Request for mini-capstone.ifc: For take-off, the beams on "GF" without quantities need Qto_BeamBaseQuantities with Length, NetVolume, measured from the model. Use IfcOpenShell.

First a look at what the model holds.

```python
import ifcopenshell
import ifcopenshell.util.element
import ifcopenshell.util.unit

model = ifcopenshell.open("mini-capstone.ifc")
print(model.schema)
for unit_type in ("LENGTHUNIT", "AREAUNIT", "VOLUMEUNIT"):
    print(unit_type, ifcopenshell.util.unit.calculate_unit_scale(model, unit_type))
storey = next(s for s in model.by_type("IfcBuildingStorey") if s.Name == "GF")
beams = [e for e in ifcopenshell.util.element.get_decomposition(storey) if e.is_a("IfcBeam")]
for e in sorted(beams, key=lambda e: e.id()):
    print(e.id(), e.is_a(), e.Name, list(ifcopenshell.util.element.get_psets(e, qtos_only=True)), sep=" | ")
```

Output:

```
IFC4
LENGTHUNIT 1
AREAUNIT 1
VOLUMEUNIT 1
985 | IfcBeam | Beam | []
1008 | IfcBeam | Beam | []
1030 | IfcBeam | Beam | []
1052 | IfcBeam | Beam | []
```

```python
import ifcopenshell
import ifcopenshell.api.pset
import ifcopenshell.geom
import ifcopenshell.util.element
import ifcopenshell.util.shape
import ifcopenshell.util.unit

model = ifcopenshell.open("mini-capstone.ifc")
unit_scale = ifcopenshell.util.unit.calculate_unit_scale(model)
volume_scale = ifcopenshell.util.unit.calculate_unit_scale(model, "VOLUMEUNIT")
settings = ifcopenshell.geom.settings()

storey = next(s for s in model.by_type("IfcBuildingStorey") if s.Name == "GF")
beams = [e for e in ifcopenshell.util.element.get_decomposition(storey) if e.is_a("IfcBeam")]

for e in sorted(beams, key=lambda e: e.id()):
    if ifcopenshell.util.element.get_psets(e, qtos_only=True, should_inherit=False):
        continue
    # Geometry comes back in metres, in the element's own axes.
    shape = ifcopenshell.geom.create_shape(settings, e)
    values = {
        "Length": ifcopenshell.util.shape.get_max_xyz(shape.geometry) / unit_scale,
        "NetVolume": ifcopenshell.util.shape.get_volume(shape.geometry) / volume_scale,
    }
    qto = ifcopenshell.api.pset.add_qto(model, product=e, name="Qto_BeamBaseQuantities")
    ifcopenshell.api.pset.edit_qto(model, qto=qto, properties=values)
    print(e.id(), {k: round(v, 3) for k, v in values.items()})

model.write("mini-capstone_edited.ifc")
```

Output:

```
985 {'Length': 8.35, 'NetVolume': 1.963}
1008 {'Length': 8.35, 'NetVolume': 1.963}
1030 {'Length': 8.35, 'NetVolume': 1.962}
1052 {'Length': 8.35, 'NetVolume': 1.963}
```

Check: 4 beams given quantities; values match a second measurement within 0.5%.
